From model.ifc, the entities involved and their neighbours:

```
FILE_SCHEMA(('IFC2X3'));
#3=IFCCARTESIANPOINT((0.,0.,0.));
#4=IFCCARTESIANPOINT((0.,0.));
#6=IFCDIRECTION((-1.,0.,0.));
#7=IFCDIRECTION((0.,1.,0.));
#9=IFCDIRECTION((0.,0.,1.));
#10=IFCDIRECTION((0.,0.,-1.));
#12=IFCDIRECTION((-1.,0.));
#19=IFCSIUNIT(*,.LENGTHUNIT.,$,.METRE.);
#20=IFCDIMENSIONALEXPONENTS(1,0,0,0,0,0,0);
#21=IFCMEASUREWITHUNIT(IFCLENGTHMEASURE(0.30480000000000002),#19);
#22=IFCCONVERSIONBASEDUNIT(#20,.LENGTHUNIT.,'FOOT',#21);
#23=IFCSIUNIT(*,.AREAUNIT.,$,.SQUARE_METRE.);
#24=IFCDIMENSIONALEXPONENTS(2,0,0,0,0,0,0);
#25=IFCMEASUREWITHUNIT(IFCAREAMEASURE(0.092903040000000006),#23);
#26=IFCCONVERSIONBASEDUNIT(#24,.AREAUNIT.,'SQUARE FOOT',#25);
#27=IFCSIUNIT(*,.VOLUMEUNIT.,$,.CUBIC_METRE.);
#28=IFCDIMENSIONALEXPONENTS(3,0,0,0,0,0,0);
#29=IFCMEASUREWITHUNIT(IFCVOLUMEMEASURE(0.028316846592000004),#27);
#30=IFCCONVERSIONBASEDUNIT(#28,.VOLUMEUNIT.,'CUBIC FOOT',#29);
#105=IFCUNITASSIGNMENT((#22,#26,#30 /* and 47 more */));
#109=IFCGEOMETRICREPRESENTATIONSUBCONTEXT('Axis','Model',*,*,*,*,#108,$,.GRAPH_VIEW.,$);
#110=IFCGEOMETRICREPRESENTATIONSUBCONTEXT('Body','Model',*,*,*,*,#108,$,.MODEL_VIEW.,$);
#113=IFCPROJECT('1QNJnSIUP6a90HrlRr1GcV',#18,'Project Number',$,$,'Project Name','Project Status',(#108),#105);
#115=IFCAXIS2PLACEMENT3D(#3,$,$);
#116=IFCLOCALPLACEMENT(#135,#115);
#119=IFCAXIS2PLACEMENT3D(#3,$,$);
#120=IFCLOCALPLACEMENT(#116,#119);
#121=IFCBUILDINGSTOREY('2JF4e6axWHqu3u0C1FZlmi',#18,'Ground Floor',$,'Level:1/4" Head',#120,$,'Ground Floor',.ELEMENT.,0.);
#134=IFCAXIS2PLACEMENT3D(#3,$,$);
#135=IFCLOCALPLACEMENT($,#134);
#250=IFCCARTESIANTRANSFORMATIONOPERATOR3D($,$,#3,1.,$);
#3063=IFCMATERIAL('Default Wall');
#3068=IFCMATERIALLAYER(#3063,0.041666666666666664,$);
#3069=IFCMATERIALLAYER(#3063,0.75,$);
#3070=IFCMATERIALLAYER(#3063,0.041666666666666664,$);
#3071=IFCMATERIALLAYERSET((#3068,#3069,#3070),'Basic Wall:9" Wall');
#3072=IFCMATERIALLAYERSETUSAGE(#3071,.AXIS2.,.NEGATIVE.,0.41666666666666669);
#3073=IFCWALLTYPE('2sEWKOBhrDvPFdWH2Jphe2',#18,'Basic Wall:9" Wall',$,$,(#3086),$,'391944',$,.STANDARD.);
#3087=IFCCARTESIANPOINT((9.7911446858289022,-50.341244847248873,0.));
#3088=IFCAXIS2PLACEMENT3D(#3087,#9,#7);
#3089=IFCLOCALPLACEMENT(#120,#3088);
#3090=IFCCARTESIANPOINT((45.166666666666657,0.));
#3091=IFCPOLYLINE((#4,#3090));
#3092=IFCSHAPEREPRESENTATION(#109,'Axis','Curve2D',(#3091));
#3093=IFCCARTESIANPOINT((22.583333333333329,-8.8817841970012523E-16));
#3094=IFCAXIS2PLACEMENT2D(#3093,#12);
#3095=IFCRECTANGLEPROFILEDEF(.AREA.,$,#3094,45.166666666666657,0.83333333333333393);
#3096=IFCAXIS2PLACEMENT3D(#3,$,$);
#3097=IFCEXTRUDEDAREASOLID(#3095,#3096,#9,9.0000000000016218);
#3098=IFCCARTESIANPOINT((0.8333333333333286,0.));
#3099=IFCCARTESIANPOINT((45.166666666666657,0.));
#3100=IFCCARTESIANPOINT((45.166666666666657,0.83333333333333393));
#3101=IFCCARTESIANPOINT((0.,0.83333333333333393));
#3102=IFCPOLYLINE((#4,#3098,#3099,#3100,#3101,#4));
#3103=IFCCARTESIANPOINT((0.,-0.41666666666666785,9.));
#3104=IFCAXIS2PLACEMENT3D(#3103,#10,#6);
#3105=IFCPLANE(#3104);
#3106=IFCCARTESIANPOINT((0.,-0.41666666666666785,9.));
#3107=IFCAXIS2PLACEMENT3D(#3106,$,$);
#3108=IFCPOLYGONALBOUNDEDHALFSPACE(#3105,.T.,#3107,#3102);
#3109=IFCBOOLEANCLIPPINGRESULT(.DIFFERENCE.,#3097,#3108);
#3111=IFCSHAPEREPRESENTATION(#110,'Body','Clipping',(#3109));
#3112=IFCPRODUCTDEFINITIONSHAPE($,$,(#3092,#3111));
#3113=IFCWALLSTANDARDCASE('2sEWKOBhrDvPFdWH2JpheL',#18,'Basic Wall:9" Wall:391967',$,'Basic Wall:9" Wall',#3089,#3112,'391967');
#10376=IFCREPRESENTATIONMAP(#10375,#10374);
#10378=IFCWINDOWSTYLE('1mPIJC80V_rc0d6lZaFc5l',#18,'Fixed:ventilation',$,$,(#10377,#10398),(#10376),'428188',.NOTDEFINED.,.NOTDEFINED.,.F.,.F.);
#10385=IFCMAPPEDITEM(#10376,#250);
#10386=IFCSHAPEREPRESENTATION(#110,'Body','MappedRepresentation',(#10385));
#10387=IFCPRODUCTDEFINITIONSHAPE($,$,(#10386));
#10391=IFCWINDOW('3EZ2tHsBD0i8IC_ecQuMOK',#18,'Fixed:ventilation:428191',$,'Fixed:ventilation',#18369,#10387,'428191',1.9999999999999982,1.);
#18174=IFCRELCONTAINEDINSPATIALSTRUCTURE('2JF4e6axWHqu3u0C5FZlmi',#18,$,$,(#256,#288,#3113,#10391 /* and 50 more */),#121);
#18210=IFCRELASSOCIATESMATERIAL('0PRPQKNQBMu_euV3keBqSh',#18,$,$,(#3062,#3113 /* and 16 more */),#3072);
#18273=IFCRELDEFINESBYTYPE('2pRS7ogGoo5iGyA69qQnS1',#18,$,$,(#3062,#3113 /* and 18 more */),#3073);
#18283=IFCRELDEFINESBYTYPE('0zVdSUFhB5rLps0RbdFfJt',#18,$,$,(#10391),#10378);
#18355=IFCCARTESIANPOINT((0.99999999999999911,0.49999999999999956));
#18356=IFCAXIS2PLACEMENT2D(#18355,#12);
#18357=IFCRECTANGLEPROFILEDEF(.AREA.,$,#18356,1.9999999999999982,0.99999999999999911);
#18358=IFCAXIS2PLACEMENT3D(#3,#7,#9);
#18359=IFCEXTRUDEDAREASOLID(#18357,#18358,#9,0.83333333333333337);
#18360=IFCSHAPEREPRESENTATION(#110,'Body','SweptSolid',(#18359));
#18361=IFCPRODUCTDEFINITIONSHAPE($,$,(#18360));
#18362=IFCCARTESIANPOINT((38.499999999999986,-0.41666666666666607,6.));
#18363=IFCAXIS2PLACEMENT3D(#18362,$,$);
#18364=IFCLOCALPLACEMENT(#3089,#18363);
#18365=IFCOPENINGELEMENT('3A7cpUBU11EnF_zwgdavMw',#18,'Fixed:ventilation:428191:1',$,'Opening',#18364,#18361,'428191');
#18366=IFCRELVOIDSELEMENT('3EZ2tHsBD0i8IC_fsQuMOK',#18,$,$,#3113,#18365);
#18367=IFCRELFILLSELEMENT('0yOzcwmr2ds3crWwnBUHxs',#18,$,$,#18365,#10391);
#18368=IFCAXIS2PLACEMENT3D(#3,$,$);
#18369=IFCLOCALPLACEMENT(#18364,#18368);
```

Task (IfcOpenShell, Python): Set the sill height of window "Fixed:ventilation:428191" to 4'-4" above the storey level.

```python
import numpy as np
import ifcopenshell
import ifcopenshell.api.geometry
import ifcopenshell.geom
import ifcopenshell.util.element
import ifcopenshell.util.placement
import ifcopenshell.util.shape
import ifcopenshell.util.unit

model = ifcopenshell.open("model.ifc")
unit_scale = ifcopenshell.util.unit.calculate_unit_scale(model)

window = model.by_guid("3EZ2tHsBD0i8IC_ecQuMOK")
opening = window.FillsVoids[0].RelatingOpeningElement
storey = ifcopenshell.util.element.get_container(window, ifc_class="IfcBuildingStorey")
level = ifcopenshell.util.placement.get_local_placement(storey.ObjectPlacement)[2, 3]

# The opening's origin need not be at the sill, so measure its lowest point.
shape = ifcopenshell.geom.create_shape(ifcopenshell.geom.settings(), opening)
bottom = ifcopenshell.util.shape.get_shape_bottom_elevation(shape, shape.geometry) / unit_scale
dz = level + 52 * 0.0254 / unit_scale - bottom

shift = np.array([0.0, 0.0, dz])
# The window is placed relative to its opening, so it follows when the opening moves.
matrix = ifcopenshell.util.placement.get_local_placement(opening.ObjectPlacement)
matrix[:3, 3] += shift
ifcopenshell.api.geometry.edit_object_placement(
    model, product=opening, matrix=matrix, is_si=False, should_transform_children=True
)

print(f"moved by {dz * unit_scale:+.3f} m")

model.write("model_updated.ifc")
```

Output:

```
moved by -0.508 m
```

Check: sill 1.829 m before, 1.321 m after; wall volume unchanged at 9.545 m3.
